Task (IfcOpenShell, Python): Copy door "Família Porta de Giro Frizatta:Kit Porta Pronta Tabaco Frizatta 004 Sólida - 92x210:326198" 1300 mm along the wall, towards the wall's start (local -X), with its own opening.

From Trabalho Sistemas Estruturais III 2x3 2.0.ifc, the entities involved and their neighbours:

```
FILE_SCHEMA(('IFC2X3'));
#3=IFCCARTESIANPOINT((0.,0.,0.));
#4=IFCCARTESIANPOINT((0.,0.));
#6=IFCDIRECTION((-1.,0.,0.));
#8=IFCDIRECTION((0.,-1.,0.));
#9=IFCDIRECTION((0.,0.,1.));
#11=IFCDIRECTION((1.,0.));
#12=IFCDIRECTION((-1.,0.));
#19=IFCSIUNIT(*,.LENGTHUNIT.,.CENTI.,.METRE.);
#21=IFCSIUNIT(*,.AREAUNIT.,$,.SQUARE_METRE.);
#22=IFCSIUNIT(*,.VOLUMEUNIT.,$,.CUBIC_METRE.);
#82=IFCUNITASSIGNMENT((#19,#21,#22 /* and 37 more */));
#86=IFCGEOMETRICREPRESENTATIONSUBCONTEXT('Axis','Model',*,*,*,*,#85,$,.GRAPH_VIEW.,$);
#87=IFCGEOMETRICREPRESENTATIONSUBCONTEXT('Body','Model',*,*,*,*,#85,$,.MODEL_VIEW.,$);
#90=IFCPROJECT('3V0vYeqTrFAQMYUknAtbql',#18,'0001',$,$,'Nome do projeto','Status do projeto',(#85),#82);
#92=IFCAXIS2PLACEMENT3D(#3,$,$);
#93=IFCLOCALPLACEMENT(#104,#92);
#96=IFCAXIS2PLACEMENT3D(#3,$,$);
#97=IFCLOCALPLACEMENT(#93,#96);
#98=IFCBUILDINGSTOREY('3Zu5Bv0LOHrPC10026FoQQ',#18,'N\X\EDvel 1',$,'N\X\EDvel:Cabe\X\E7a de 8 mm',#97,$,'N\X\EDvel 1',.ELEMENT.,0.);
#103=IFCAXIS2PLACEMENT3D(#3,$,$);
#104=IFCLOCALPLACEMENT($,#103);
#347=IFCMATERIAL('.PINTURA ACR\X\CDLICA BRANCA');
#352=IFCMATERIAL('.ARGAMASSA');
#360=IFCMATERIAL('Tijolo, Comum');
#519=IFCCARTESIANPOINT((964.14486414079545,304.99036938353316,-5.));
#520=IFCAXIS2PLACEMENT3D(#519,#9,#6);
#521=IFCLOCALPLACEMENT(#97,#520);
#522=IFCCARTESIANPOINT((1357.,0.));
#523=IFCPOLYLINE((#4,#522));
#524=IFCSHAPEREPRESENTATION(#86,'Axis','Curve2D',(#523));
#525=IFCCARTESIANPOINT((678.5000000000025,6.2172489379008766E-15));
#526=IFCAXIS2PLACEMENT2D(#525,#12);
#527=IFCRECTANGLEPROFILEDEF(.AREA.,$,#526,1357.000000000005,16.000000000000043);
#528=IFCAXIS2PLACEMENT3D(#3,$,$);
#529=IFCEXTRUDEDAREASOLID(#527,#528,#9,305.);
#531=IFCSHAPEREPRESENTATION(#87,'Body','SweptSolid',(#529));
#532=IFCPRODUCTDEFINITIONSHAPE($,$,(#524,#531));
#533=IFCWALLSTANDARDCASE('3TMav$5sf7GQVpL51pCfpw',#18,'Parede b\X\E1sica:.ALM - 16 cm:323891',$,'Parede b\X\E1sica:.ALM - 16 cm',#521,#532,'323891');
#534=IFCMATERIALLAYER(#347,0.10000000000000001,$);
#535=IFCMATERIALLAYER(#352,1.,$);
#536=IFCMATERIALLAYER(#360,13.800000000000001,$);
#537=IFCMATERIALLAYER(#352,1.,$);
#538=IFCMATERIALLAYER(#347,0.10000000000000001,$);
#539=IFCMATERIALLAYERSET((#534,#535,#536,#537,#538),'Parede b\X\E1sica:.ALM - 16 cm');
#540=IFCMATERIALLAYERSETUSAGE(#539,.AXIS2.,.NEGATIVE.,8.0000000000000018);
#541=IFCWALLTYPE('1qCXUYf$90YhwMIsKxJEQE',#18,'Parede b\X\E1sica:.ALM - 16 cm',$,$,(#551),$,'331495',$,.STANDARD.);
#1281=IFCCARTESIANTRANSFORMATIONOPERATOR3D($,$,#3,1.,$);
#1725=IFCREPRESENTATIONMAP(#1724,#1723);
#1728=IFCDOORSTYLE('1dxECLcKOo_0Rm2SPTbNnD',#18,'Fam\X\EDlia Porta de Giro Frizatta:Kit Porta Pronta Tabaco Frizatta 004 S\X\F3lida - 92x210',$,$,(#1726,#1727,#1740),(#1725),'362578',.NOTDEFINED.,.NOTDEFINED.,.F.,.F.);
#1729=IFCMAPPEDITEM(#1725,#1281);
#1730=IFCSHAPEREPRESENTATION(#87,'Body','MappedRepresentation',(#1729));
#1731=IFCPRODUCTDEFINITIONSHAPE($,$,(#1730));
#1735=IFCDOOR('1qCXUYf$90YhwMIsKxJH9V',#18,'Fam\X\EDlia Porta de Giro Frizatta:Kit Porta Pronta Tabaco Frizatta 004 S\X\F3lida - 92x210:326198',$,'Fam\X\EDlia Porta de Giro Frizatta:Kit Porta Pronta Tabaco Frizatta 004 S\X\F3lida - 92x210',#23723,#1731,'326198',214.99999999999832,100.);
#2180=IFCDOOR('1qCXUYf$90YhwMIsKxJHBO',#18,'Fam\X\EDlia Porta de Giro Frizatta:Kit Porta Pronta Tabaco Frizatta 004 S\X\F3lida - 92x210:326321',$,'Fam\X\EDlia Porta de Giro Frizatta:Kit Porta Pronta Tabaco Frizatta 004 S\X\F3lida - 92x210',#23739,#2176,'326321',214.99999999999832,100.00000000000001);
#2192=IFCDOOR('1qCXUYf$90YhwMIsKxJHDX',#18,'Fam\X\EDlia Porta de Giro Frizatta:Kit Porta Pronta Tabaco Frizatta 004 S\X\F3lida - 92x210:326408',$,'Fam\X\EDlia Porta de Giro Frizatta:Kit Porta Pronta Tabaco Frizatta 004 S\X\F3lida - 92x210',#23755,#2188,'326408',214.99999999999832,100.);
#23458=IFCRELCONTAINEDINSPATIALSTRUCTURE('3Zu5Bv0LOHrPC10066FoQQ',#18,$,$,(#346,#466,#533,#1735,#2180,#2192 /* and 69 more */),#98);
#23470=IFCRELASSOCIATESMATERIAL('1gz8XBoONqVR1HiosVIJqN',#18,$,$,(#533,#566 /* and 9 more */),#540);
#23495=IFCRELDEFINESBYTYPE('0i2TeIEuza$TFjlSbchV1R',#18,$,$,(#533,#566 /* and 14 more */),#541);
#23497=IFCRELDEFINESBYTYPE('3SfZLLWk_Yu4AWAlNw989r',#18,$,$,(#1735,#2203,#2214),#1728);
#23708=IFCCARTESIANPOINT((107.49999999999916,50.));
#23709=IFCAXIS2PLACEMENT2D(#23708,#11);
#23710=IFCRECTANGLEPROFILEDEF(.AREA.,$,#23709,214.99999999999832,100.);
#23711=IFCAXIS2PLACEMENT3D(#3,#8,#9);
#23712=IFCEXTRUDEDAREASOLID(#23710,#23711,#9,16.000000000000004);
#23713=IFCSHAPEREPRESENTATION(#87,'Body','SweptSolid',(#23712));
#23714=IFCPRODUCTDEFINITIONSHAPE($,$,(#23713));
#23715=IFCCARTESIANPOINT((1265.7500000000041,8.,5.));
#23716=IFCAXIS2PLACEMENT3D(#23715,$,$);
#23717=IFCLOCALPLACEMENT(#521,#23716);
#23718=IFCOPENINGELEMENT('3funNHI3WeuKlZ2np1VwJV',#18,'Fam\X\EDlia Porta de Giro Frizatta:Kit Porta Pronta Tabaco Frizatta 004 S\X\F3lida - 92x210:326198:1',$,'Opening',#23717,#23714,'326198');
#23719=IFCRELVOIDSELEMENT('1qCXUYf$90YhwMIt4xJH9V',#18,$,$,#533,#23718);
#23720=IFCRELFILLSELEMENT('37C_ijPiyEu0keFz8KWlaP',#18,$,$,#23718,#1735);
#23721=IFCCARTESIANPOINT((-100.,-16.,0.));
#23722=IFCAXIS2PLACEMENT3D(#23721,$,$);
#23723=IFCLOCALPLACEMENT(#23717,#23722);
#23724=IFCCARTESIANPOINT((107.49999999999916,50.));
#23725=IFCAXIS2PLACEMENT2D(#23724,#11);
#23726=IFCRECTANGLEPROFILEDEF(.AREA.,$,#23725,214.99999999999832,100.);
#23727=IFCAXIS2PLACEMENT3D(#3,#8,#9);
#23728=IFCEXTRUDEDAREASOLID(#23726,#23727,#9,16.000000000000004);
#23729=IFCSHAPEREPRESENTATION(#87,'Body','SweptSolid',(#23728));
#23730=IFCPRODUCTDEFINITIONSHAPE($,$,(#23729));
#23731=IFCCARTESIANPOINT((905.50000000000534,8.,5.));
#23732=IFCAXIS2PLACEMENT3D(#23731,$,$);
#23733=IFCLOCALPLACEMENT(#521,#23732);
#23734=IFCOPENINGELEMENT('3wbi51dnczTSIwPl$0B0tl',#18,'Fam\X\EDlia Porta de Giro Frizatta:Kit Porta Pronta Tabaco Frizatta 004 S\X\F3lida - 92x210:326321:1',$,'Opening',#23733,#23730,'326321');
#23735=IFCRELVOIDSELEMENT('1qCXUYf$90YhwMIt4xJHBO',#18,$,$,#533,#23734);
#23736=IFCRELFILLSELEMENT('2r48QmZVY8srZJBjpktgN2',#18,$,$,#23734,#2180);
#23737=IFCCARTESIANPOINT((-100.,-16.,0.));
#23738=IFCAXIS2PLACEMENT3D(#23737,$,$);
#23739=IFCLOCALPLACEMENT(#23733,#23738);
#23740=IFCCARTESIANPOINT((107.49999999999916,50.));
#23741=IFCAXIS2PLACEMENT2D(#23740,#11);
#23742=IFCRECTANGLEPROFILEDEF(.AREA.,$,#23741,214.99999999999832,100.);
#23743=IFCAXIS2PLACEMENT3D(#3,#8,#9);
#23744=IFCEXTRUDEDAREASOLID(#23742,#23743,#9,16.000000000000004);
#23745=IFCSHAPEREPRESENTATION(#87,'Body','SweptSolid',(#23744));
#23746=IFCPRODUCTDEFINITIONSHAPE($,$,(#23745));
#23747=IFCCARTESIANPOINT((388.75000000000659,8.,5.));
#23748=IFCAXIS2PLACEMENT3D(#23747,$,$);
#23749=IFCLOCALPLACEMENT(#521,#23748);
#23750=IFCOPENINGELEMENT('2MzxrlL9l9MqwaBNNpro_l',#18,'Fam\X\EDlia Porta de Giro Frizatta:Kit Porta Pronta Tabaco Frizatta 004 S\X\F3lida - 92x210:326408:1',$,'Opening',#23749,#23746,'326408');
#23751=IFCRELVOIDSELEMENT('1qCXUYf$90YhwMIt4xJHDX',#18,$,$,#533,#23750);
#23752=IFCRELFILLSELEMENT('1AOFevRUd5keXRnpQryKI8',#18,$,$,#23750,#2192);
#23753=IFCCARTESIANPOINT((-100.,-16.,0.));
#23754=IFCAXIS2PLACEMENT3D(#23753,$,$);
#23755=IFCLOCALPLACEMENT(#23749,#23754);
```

```python
import ifcopenshell
import ifcopenshell.api.feature
import ifcopenshell.api.geometry
import ifcopenshell.api.root
import ifcopenshell.geom
import ifcopenshell.util.element
import ifcopenshell.util.placement
import ifcopenshell.util.shape
import ifcopenshell.util.unit

model = ifcopenshell.open("Trabalho Sistemas Estruturais III 2x3 2.0.ifc")
unit_scale = ifcopenshell.util.unit.calculate_unit_scale(model)
settings = ifcopenshell.geom.settings()


def volume(element):
    """Net volume in cubic metres, openings subtracted."""
    shape = ifcopenshell.geom.create_shape(settings, element)
    return ifcopenshell.util.shape.get_volume(shape.geometry)


def reuse_history(source, copy):
    """copy_class also copies each property set's owner history, people and application; keep the originals."""
    for rel in copy.IsDefinedBy:
        if rel.is_a("IfcRelDefinesByProperties") and (history := rel.RelatingPropertyDefinition.OwnerHistory):
            rel.RelatingPropertyDefinition.OwnerHistory = source.OwnerHistory
            ifcopenshell.util.element.remove_deep2(model, history)


door = model.by_guid("1qCXUYf$90YhwMIsKxJH9V")
opening = door.FillsVoids[0].RelatingOpeningElement
wall = opening.VoidsElements[0].RelatingBuildingElement
before = volume(wall)
shift = ifcopenshell.util.placement.get_local_placement(wall.ObjectPlacement)[:3, 0] * -1.3 / unit_scale

# copy_class copies the void relationship, type, container and properties, but no geometry.
new_opening = ifcopenshell.api.root.copy_class(model, product=opening)
new_opening.Representation = ifcopenshell.util.element.copy_deep(
    model, opening.Representation, exclude=["IfcGeometricRepresentationContext", "IfcRepresentationMap"]
)
new_opening.Name = "Família Porta de Giro Frizatta:Kit Porta Pronta Tabaco Frizatta 004 Sólida - 92x210"
new_opening.Tag = None
new_door = ifcopenshell.api.root.copy_class(model, product=door)
new_door.Representation = ifcopenshell.util.element.copy_deep(
    model, door.Representation, exclude=["IfcGeometricRepresentationContext", "IfcRepresentationMap"]
)
new_door.Name = "Família Porta de Giro Frizatta:Kit Porta Pronta Tabaco Frizatta 004 Sólida - 92x210"
new_door.Tag = None
reuse_history(door, new_door)
fills = ifcopenshell.api.feature.add_filling(model, opening=new_opening, element=new_door)
fills.OwnerHistory = new_door.OwnerHistory  # required in IFC2X3

for old, new in ((opening, new_opening), (door, new_door)):
    matrix = ifcopenshell.util.placement.get_local_placement(old.ObjectPlacement)
    matrix[:3, 3] += shift
    ifcopenshell.api.geometry.edit_object_placement(model, product=new, matrix=matrix, is_si=False)

after = volume(wall)

print(f"wall volume {before:.3f} -> {after:.3f} m3")

model.write("Trabalho Sistemas Estruturais III 2x3 2.0_v2.ifc")
```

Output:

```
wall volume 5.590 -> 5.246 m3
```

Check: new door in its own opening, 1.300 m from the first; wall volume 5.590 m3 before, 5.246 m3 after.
